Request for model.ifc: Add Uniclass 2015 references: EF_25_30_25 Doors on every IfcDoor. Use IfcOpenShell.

First a look at what the model holds.

```python
import ifcopenshell

model = ifcopenshell.open("model.ifc")
print(model.schema)
print("classifications:", [c.Name for c in model.by_type("IfcClassification")])
for ifc_class in ("IfcDoor", "IfcRoof", "IfcStair", "IfcWall", "IfcWindow"):
    print(ifc_class, len(model.by_type(ifc_class)))
```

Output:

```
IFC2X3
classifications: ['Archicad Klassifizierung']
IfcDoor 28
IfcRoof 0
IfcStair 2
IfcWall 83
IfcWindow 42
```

```python
import ifcopenshell
import ifcopenshell.api.classification

model = ifcopenshell.open("model.ifc")

# IFC2X3 requires Source and Edition and has no link from the project to the system.
system = model.create_entity("IfcClassification", Source="NBS", Edition="2015", Name="Uniclass 2015")

codes = {
    "IfcDoor": ("EF_25_30_25", "Doors"),
}
for ifc_class, (code, name) in codes.items():
    products = model.by_type(ifc_class)
    ifcopenshell.api.classification.add_reference(
        model, products=products, classification=system, identification=code, name=name
    )
    print(code, len(products))

model.write("model_edited.ifc")
```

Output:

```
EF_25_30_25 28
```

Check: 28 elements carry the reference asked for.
